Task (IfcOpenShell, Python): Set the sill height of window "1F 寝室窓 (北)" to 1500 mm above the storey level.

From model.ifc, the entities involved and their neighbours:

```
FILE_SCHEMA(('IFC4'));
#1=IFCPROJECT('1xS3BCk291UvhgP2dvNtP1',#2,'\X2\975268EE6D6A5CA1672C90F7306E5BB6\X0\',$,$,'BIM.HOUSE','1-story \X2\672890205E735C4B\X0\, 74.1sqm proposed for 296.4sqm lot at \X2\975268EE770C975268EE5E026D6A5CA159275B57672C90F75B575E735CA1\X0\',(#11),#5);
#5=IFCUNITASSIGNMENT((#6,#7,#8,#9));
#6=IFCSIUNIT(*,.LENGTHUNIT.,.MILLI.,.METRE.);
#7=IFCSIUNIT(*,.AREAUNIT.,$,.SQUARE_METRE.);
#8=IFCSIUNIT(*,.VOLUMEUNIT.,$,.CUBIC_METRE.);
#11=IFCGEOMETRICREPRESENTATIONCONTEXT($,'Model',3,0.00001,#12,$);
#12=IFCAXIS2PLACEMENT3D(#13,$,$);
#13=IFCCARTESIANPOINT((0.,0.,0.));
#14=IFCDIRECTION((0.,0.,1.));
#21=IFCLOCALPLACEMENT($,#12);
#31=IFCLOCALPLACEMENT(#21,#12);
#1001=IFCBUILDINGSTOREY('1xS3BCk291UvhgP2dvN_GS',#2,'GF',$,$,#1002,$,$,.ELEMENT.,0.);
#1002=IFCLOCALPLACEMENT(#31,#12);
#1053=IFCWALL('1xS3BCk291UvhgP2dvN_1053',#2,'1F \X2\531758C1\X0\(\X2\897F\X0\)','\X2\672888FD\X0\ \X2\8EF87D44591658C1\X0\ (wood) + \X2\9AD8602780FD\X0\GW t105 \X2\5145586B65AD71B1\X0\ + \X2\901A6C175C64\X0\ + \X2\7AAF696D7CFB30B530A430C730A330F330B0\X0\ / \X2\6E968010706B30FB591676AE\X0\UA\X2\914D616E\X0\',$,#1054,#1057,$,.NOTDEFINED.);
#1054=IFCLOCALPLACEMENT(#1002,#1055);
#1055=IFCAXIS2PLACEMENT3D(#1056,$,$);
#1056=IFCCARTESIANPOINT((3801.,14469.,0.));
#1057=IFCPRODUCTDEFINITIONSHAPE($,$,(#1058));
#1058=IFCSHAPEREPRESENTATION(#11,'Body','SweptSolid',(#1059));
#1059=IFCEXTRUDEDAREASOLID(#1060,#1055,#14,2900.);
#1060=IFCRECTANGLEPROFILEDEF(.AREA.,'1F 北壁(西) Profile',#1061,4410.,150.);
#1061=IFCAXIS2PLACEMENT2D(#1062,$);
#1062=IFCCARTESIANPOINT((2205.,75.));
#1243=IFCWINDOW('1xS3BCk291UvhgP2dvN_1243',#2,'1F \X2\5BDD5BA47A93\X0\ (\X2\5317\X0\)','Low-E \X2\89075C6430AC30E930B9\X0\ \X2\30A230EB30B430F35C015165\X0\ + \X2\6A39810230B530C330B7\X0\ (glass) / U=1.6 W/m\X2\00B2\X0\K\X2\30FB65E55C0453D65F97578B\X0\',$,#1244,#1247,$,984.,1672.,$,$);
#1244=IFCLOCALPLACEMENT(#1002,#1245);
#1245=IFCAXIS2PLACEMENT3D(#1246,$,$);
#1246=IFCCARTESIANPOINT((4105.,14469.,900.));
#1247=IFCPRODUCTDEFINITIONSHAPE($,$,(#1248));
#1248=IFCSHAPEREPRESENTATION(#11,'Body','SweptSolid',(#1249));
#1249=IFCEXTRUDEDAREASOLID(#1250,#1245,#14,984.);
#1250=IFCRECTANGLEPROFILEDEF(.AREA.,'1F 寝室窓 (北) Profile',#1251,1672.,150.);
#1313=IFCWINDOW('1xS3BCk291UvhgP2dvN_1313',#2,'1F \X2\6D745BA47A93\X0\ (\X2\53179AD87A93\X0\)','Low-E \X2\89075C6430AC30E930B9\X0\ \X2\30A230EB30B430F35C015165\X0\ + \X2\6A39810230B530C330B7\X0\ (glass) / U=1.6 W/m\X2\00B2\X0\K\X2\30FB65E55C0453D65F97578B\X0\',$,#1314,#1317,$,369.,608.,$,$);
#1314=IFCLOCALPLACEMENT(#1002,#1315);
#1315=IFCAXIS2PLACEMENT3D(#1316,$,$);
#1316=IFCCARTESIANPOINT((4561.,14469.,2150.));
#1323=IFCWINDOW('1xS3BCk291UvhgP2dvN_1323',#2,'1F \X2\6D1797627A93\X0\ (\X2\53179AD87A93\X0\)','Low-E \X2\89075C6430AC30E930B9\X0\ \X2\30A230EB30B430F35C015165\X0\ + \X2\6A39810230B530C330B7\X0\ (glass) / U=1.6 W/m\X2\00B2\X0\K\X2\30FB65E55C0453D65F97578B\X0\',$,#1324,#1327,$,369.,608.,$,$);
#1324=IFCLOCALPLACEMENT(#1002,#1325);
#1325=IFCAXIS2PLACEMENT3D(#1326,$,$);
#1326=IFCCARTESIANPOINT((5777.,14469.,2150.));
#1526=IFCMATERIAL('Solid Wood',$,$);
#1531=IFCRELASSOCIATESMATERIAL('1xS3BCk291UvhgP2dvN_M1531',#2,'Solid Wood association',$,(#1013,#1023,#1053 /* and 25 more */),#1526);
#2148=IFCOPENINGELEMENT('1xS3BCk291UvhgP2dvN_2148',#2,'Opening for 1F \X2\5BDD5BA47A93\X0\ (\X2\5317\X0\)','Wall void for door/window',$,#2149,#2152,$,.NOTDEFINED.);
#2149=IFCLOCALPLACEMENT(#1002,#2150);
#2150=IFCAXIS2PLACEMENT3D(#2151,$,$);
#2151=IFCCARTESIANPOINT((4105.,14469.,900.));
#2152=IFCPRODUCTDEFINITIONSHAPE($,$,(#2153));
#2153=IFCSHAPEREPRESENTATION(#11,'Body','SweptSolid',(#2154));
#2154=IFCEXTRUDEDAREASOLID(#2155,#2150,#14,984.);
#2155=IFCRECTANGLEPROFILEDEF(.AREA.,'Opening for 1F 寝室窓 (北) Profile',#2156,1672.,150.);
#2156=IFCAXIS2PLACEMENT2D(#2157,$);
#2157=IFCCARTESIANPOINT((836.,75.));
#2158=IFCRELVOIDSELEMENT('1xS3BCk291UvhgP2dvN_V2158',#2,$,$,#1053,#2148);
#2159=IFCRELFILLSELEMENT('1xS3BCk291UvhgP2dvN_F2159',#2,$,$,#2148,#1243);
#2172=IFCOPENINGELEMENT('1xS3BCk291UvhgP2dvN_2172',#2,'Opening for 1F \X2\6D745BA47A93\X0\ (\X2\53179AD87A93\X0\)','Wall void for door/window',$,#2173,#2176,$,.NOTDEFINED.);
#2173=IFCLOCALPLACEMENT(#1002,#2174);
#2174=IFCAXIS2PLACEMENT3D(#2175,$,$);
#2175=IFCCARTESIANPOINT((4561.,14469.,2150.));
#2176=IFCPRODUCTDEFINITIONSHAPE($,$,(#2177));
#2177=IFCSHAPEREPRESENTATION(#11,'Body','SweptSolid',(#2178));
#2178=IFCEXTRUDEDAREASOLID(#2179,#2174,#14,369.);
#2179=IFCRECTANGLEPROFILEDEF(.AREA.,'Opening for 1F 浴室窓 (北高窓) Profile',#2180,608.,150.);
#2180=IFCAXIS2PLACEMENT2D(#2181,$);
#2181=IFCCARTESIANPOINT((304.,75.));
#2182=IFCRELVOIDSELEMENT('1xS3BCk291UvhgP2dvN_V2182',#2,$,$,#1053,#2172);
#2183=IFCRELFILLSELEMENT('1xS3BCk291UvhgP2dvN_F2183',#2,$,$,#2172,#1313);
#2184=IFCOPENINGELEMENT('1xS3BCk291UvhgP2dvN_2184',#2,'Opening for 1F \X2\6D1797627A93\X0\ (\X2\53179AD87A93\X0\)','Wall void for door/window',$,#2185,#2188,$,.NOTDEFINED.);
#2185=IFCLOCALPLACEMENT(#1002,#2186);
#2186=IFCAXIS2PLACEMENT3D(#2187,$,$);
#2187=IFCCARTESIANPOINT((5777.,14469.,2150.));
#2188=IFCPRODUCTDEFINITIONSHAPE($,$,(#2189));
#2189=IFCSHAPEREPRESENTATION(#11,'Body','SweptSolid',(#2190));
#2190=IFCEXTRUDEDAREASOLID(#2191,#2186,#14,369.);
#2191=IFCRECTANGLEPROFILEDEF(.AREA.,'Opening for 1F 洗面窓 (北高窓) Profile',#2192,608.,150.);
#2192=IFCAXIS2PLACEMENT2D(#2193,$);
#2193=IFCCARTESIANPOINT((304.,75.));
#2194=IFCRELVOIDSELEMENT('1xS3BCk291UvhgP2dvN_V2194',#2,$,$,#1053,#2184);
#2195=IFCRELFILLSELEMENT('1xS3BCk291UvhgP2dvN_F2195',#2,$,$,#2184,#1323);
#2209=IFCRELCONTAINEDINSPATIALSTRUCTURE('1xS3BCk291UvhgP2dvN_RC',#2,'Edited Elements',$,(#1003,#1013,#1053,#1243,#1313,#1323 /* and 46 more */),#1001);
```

```python
import numpy as np
import ifcopenshell
import ifcopenshell.api.geometry
import ifcopenshell.geom
import ifcopenshell.util.element
import ifcopenshell.util.placement
import ifcopenshell.util.shape
import ifcopenshell.util.unit

model = ifcopenshell.open("model.ifc")
unit_scale = ifcopenshell.util.unit.calculate_unit_scale(model)

window = model.by_id(1243)
opening = window.FillsVoids[0].RelatingOpeningElement
storey = ifcopenshell.util.element.get_container(window, ifc_class="IfcBuildingStorey")
level = ifcopenshell.util.placement.get_local_placement(storey.ObjectPlacement)[2, 3]

# The opening's origin need not be at the sill, so measure its lowest point.
shape = ifcopenshell.geom.create_shape(ifcopenshell.geom.settings(), opening)
bottom = ifcopenshell.util.shape.get_shape_bottom_elevation(shape, shape.geometry) / unit_scale
dz = level + 1500.0 - bottom

shift = np.array([0.0, 0.0, dz])
# The window is not placed relative to its opening, so move both.
for product in (opening, window):
    matrix = ifcopenshell.util.placement.get_local_placement(product.ObjectPlacement)
    matrix[:3, 3] += shift
    ifcopenshell.api.geometry.edit_object_placement(model, product=product, matrix=matrix, is_si=False)

print(f"moved by {dz * unit_scale:+.3f} m")

model.write("model_updated.ifc")
```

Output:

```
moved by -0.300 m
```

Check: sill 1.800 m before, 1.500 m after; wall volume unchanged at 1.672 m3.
